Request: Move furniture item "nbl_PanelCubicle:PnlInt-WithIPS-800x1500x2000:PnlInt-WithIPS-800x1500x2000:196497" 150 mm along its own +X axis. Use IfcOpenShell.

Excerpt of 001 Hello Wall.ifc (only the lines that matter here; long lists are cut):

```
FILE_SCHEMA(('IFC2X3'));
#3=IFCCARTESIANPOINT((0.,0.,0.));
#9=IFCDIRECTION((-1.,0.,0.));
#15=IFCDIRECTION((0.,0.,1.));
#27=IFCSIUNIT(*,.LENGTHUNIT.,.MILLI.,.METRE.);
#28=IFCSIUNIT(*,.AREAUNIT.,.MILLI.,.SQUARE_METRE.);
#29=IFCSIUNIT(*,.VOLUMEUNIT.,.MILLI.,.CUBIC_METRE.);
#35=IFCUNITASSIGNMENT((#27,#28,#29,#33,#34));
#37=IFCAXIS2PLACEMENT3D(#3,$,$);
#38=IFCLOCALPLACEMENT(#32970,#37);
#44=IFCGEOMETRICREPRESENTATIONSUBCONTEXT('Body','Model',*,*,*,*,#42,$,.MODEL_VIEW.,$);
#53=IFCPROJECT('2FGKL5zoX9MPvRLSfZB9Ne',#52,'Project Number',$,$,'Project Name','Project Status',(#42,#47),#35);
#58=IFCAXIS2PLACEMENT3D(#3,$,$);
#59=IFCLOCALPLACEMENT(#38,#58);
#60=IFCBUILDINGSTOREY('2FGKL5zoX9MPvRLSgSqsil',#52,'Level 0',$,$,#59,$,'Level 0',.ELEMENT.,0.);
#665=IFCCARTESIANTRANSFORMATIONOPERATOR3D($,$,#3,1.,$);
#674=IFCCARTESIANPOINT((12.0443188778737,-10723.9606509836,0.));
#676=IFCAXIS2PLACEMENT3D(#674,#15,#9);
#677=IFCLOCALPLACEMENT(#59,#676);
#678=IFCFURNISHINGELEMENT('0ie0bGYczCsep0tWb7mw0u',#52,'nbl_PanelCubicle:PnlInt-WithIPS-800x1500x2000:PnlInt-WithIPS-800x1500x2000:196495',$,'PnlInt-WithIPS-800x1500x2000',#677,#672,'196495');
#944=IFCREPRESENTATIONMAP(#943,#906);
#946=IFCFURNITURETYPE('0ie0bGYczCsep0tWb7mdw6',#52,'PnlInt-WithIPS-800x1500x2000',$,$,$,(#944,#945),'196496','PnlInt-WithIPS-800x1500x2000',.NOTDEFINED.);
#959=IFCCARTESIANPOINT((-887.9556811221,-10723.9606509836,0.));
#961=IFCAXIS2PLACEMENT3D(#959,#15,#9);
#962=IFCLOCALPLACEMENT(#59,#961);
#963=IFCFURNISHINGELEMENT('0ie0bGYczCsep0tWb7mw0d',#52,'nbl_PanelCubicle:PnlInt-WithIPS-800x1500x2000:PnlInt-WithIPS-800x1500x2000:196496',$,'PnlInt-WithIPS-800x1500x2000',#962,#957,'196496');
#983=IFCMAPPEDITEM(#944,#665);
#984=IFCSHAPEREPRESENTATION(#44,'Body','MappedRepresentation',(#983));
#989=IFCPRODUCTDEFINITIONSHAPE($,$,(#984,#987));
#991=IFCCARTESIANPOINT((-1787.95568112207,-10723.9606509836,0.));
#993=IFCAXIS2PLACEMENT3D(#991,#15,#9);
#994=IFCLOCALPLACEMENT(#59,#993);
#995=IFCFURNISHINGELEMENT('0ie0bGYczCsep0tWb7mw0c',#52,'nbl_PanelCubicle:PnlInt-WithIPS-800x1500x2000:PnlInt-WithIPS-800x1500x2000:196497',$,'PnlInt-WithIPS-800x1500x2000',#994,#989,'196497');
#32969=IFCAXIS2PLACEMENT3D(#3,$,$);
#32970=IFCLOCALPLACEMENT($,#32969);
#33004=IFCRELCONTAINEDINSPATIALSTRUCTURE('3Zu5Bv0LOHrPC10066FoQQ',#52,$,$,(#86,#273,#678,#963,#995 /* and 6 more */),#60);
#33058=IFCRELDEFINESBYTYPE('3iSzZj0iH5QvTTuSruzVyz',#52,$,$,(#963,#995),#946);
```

```python
import ifcopenshell
import ifcopenshell.api.geometry
import ifcopenshell.util.placement

model = ifcopenshell.open("001 Hello Wall.ifc")

item = model.by_guid("0ie0bGYczCsep0tWb7mw0c")
matrix = ifcopenshell.util.placement.get_local_placement(item.ObjectPlacement)
matrix[:3, 3] += matrix[:3, 0] * 150.0
ifcopenshell.api.geometry.edit_object_placement(model, product=item, matrix=matrix, is_si=False)

print(ifcopenshell.util.placement.get_local_placement(item.ObjectPlacement).round(3) + 0.0)

model.write("001 Hello Wall-out.ifc")
```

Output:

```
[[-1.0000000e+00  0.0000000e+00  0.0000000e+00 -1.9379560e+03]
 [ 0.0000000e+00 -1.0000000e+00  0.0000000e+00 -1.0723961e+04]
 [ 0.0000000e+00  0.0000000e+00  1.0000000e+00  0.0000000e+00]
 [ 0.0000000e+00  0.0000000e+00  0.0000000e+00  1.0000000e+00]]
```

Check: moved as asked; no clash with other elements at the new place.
